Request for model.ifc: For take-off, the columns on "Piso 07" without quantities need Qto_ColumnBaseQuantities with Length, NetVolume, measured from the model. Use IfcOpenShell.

First a look at what the model holds.

```python
import ifcopenshell
import ifcopenshell.util.element
import ifcopenshell.util.unit

model = ifcopenshell.open("model.ifc")
print(model.schema)
for unit_type in ("LENGTHUNIT", "AREAUNIT", "VOLUMEUNIT"):
    print(unit_type, ifcopenshell.util.unit.calculate_unit_scale(model, unit_type))
storey = next(s for s in model.by_type("IfcBuildingStorey") if s.Name == "Piso 07")
columns = [e for e in ifcopenshell.util.element.get_decomposition(storey) if e.is_a("IfcColumn")]
for e in sorted(columns, key=lambda e: e.id()):
    print(e.id(), e.is_a(), e.Name, list(ifcopenshell.util.element.get_psets(e, qtos_only=True)), sep=" | ")
```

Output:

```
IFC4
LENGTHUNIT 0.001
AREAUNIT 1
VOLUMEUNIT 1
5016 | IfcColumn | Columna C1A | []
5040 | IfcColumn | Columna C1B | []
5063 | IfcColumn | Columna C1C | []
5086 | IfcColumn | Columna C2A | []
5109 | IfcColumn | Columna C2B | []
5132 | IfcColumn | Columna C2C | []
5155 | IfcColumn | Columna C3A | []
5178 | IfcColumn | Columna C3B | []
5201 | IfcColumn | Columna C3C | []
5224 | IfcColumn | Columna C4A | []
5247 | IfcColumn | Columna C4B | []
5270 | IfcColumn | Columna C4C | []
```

```python
import ifcopenshell
import ifcopenshell.api.pset
import ifcopenshell.geom
import ifcopenshell.util.element
import ifcopenshell.util.shape
import ifcopenshell.util.unit

model = ifcopenshell.open("model.ifc")
unit_scale = ifcopenshell.util.unit.calculate_unit_scale(model)
volume_scale = ifcopenshell.util.unit.calculate_unit_scale(model, "VOLUMEUNIT")
settings = ifcopenshell.geom.settings()

storey = next(s for s in model.by_type("IfcBuildingStorey") if s.Name == "Piso 07")
columns = [e for e in ifcopenshell.util.element.get_decomposition(storey) if e.is_a("IfcColumn")]

for e in sorted(columns, key=lambda e: e.id()):
    if ifcopenshell.util.element.get_psets(e, qtos_only=True, should_inherit=False):
        continue
    # Geometry comes back in metres, in the element's own axes.
    shape = ifcopenshell.geom.create_shape(settings, e)
    values = {
        "Length": ifcopenshell.util.shape.get_z(shape.geometry) / unit_scale,
        "NetVolume": ifcopenshell.util.shape.get_volume(shape.geometry) / volume_scale,
    }
    qto = ifcopenshell.api.pset.add_qto(model, product=e, name="Qto_ColumnBaseQuantities")
    ifcopenshell.api.pset.edit_qto(model, qto=qto, properties=values)
    print(e.id(), {k: round(v, 3) for k, v in values.items()})

model.write("model_v2.ifc")
```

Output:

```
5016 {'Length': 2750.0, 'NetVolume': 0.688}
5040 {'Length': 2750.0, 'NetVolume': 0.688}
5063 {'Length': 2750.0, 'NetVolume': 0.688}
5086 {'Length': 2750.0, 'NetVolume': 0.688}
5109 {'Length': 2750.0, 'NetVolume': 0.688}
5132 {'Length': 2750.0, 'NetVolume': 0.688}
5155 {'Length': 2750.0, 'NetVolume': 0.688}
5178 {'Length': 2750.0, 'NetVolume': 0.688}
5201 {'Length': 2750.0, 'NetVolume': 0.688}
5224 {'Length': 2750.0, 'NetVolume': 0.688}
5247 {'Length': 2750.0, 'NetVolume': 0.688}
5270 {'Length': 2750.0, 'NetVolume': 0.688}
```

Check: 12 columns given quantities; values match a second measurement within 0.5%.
